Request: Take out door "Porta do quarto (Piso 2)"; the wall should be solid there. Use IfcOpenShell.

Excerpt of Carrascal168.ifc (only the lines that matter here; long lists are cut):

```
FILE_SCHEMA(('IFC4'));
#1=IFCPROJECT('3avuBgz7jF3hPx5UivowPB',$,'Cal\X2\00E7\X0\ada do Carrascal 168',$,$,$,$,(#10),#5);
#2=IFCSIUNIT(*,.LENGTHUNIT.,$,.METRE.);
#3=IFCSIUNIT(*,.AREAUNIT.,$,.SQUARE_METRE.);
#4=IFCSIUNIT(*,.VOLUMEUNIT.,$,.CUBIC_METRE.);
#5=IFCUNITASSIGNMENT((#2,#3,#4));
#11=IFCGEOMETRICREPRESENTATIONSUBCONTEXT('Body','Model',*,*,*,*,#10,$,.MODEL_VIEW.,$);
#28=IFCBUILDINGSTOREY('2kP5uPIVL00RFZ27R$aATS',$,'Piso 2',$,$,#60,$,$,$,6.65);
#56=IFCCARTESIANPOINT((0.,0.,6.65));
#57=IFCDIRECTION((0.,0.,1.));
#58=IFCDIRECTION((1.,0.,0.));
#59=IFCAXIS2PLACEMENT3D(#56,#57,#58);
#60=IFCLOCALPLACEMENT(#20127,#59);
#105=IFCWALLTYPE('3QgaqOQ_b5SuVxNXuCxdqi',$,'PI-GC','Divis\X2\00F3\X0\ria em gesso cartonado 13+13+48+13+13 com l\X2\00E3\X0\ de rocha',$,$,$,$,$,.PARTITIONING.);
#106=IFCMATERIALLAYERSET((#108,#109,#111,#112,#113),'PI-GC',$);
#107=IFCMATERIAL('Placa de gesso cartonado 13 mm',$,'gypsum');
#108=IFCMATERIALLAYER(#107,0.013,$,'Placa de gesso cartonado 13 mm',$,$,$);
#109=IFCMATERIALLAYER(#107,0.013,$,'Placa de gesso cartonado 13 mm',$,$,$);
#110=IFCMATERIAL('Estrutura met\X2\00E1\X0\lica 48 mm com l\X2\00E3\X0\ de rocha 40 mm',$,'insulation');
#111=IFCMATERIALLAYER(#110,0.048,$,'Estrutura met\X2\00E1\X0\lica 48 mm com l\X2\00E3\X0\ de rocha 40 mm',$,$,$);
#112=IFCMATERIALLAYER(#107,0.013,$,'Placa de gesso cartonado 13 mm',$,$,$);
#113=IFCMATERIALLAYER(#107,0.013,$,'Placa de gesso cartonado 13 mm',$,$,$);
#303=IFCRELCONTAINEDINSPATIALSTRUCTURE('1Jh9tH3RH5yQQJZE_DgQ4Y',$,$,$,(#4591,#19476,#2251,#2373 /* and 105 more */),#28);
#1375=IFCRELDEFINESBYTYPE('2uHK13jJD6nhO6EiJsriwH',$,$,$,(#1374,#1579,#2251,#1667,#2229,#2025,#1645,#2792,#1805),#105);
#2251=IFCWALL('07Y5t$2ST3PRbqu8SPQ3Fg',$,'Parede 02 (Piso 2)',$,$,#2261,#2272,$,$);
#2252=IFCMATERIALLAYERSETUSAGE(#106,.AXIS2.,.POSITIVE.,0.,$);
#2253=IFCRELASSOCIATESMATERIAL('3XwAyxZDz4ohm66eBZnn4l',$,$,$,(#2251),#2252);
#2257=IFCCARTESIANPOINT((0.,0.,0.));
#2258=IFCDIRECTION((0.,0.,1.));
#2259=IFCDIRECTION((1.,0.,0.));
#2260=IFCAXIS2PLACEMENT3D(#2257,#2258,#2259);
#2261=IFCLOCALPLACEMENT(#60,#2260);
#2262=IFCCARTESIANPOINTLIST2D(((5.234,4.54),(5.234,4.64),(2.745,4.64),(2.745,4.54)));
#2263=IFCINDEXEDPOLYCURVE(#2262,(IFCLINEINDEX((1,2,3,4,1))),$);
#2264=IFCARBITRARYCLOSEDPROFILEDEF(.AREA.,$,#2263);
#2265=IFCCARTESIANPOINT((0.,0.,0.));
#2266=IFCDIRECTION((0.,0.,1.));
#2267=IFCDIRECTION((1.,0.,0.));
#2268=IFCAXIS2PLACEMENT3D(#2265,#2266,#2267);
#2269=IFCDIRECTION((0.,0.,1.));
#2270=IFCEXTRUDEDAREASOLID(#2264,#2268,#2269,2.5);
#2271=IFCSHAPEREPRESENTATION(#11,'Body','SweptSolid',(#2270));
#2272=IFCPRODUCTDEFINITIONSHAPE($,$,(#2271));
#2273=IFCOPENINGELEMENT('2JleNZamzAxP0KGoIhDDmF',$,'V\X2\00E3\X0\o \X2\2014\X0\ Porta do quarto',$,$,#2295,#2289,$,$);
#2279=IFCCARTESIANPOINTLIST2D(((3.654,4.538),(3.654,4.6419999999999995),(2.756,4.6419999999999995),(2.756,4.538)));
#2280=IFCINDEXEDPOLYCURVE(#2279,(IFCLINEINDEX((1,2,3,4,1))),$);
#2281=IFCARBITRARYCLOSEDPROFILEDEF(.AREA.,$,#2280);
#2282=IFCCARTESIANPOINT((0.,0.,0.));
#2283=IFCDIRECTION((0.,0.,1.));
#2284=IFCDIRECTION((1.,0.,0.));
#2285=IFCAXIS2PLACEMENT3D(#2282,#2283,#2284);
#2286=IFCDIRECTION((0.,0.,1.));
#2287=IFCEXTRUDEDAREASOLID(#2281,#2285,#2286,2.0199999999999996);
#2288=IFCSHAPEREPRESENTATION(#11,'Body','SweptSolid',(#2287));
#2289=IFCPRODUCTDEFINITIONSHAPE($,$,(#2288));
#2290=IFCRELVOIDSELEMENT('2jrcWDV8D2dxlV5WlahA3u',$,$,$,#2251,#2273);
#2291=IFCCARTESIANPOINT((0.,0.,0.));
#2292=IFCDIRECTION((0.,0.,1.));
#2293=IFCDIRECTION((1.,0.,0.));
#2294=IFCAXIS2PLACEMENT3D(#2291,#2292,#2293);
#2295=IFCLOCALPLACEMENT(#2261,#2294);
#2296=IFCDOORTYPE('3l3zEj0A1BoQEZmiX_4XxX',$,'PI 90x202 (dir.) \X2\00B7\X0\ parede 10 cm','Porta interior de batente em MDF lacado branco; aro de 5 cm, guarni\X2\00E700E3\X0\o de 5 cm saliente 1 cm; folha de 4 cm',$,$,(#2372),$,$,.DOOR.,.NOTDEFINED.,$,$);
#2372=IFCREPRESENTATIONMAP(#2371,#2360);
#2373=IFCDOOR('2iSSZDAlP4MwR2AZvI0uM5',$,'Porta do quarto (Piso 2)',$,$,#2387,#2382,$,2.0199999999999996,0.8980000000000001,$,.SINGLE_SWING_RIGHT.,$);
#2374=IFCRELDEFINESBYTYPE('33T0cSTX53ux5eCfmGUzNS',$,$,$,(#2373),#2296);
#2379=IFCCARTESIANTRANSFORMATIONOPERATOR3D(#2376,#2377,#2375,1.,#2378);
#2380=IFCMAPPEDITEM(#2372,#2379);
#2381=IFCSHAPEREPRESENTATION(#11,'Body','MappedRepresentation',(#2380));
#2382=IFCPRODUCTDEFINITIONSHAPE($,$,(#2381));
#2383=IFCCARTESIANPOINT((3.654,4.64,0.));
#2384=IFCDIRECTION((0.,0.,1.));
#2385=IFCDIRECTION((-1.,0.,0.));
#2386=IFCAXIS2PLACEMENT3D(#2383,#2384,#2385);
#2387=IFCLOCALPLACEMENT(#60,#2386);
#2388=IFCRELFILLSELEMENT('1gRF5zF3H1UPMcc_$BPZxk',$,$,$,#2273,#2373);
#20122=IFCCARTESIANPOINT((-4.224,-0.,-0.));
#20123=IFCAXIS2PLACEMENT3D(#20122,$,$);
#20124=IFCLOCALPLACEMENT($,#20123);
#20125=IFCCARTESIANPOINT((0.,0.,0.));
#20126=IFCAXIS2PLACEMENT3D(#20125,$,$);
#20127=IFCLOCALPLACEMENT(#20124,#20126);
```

```python
import ifcopenshell
import ifcopenshell.api.feature
import ifcopenshell.api.root
import ifcopenshell.geom
import ifcopenshell.util.shape

model = ifcopenshell.open("Carrascal168.ifc")
settings = ifcopenshell.geom.settings()


def volume(element):
    """Net volume in cubic metres, openings subtracted."""
    shape = ifcopenshell.geom.create_shape(settings, element)
    return ifcopenshell.util.shape.get_volume(shape.geometry)


door = model.by_guid("2iSSZDAlP4MwR2AZvI0uM5")
opening = door.FillsVoids[0].RelatingOpeningElement
wall = opening.VoidsElements[0].RelatingBuildingElement
before = volume(wall)

ifcopenshell.api.root.remove_product(model, product=door)
ifcopenshell.api.feature.remove_feature(model, feature=opening)

after = volume(wall)

print(f"wall volume {before:.3f} -> {after:.3f} m3")

model.write("Carrascal168-out.ifc")
```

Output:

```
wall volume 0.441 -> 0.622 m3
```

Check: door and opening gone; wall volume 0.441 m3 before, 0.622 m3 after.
